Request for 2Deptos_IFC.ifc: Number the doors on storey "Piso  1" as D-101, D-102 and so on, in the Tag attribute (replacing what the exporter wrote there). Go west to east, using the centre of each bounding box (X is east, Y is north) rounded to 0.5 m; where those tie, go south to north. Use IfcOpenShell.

First a look at what the model holds.

```python
import ifcopenshell
import ifcopenshell.util.element
import ifcopenshell.util.placement

model = ifcopenshell.open("2Deptos_IFC.ifc")
print(model.schema)
storey = next(s for s in model.by_type("IfcBuildingStorey") if s.Name == "Piso  1")
doors = [e for e in ifcopenshell.util.element.get_decomposition(storey) if e.is_a("IfcDoor")]
for e in sorted(doors, key=lambda e: e.id()):
    origin = ifcopenshell.util.placement.get_local_placement(e.ObjectPlacement)[:3, 3]
    print(e.id(), e.Tag, e.Name, origin.round(2) + 0.0, sep=" | ")
```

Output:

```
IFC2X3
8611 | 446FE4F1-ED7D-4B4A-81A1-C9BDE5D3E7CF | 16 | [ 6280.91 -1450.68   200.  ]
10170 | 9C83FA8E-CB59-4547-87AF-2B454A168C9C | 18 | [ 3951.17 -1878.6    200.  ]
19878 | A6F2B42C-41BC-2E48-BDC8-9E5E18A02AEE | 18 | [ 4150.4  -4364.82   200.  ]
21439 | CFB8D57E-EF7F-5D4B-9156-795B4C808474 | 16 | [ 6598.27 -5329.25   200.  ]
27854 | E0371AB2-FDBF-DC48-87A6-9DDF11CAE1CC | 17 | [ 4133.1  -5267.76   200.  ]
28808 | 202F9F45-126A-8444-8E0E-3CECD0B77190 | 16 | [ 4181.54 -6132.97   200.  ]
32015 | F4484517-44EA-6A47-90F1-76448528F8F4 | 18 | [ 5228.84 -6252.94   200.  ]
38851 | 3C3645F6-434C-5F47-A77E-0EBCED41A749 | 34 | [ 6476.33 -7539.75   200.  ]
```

```python
import ifcopenshell
import ifcopenshell.geom
import ifcopenshell.util.element
import ifcopenshell.util.shape

model = ifcopenshell.open("2Deptos_IFC.ifc")
settings = ifcopenshell.geom.settings()
settings.set("use-world-coords", True)


def centre(element):
    shape = ifcopenshell.geom.create_shape(settings, element)
    return ifcopenshell.util.shape.get_bbox_centroid(shape.geometry)


storey = next(s for s in model.by_type("IfcBuildingStorey") if s.Name == "Piso  1")
doors = [e for e in ifcopenshell.util.element.get_decomposition(storey) if e.is_a("IfcDoor")]

# Insertion points can sit at a corner or the storey origin, so sort by the geometry (in metres).
centres = {e: centre(e) for e in doors}
doors.sort(key=lambda e: (round(centres[e][0] / 0.5), centres[e][1]))

for i, e in enumerate(doors, start=1):
    number = f"D-1{i:02d}"
    e.Tag = number
    print(e.id(), number)

model.write("2Deptos_IFC_updated.ifc")
```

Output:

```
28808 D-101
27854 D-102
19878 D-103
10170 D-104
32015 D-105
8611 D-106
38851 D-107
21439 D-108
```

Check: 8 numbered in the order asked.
